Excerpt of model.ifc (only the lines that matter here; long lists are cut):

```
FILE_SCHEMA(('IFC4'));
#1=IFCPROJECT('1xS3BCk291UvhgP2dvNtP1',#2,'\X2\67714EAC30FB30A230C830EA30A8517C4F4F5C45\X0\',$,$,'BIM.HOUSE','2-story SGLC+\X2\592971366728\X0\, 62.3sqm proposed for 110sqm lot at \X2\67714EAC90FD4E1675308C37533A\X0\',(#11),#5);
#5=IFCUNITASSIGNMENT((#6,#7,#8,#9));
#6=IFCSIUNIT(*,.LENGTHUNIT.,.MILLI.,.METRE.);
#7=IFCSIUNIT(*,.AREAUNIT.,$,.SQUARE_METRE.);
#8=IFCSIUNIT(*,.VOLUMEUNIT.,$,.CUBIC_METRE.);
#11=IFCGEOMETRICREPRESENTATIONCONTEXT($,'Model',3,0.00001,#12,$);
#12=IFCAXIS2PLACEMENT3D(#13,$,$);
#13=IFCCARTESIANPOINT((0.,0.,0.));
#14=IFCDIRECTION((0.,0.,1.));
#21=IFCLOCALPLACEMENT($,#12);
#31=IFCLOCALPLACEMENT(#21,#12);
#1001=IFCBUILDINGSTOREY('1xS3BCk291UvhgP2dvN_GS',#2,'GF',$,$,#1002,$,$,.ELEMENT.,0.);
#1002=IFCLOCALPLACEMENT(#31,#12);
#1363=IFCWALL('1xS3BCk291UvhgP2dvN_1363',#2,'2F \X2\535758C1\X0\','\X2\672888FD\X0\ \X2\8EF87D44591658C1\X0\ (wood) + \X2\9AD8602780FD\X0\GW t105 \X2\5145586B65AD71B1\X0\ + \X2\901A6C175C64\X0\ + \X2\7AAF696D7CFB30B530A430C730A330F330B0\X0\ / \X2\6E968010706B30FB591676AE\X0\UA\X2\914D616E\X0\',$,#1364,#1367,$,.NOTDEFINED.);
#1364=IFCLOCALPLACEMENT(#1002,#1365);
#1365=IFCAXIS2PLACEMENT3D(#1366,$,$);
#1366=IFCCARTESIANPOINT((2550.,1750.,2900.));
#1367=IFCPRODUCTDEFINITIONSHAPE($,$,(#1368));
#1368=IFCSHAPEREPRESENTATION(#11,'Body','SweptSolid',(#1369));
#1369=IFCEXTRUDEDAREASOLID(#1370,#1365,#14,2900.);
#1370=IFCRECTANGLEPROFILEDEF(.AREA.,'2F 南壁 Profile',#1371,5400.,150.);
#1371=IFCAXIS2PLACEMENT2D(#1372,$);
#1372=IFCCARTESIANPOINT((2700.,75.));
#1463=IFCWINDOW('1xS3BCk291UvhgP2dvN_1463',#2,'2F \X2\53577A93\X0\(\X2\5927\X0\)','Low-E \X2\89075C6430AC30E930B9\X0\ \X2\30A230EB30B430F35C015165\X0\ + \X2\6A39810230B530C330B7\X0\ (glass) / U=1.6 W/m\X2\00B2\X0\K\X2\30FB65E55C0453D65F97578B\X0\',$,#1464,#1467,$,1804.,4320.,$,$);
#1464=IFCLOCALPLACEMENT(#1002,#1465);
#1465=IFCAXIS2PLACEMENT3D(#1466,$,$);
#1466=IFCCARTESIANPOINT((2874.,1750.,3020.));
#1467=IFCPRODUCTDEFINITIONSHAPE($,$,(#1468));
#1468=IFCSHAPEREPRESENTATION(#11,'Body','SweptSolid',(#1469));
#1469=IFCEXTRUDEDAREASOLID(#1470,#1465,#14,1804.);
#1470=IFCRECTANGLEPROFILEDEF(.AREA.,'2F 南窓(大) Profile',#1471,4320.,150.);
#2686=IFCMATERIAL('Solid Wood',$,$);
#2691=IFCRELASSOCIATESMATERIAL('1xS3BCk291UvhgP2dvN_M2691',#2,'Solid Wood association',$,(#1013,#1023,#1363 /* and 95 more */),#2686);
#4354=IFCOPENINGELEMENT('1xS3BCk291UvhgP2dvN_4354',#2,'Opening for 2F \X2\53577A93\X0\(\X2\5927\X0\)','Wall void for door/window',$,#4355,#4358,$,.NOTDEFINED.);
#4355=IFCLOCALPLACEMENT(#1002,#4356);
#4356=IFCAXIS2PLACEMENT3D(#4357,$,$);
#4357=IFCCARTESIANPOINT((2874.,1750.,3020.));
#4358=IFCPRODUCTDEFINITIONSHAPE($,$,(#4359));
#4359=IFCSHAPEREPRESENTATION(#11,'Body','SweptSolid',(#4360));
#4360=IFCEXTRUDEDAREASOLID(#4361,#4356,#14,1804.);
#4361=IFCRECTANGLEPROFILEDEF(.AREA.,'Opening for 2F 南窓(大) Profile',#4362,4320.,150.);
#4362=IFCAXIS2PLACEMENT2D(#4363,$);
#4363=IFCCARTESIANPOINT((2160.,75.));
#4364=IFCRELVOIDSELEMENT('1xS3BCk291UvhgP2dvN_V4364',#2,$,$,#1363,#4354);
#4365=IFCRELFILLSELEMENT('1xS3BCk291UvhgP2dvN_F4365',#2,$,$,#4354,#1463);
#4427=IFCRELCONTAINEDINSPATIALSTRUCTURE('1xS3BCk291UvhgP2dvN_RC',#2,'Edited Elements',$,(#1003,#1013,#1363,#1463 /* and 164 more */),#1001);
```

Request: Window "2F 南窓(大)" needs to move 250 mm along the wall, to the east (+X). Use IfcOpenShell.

```python
import ifcopenshell
import ifcopenshell.api.geometry
import ifcopenshell.util.placement
import ifcopenshell.util.unit

model = ifcopenshell.open("model.ifc")
unit_scale = ifcopenshell.util.unit.calculate_unit_scale(model)

window = model.by_id(1463)
opening = window.FillsVoids[0].RelatingOpeningElement
wall = opening.VoidsElements[0].RelatingBuildingElement

wall_matrix = ifcopenshell.util.placement.get_local_placement(wall.ObjectPlacement)
shift = wall_matrix[:3, 0] * 0.25 / unit_scale
before = ifcopenshell.util.placement.get_local_placement(window.ObjectPlacement)[:3, 3].copy()

# The window is not placed relative to its opening, so move both.
for product in (opening, window):
    matrix = ifcopenshell.util.placement.get_local_placement(product.ObjectPlacement)
    matrix[:3, 3] += shift
    ifcopenshell.api.geometry.edit_object_placement(model, product=product, matrix=matrix, is_si=False)

after = ifcopenshell.util.placement.get_local_placement(window.ObjectPlacement)[:3, 3]
print("window moved by", (after - before).round(3) + 0.0)

model.write("model_rev.ifc")
```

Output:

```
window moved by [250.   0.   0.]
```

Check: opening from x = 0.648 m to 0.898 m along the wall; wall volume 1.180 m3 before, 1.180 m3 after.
